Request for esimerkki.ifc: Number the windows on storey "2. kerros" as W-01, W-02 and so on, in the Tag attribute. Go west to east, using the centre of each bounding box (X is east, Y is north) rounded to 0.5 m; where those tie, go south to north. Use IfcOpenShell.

First a look at what the model holds.

```python
import ifcopenshell
import ifcopenshell.util.element
import ifcopenshell.util.placement

model = ifcopenshell.open("esimerkki.ifc")
print(model.schema)
storey = next(s for s in model.by_type("IfcBuildingStorey") if s.Name == "2. kerros")
windows = [e for e in ifcopenshell.util.element.get_decomposition(storey) if e.is_a("IfcWindow")]
for e in sorted(windows, key=lambda e: e.id()):
    origin = ifcopenshell.util.placement.get_local_placement(e.ObjectPlacement)[:3, 3]
    print(e.id(), e.Tag, e.Name, origin.round(2) + 0.0, sep=" | ")
```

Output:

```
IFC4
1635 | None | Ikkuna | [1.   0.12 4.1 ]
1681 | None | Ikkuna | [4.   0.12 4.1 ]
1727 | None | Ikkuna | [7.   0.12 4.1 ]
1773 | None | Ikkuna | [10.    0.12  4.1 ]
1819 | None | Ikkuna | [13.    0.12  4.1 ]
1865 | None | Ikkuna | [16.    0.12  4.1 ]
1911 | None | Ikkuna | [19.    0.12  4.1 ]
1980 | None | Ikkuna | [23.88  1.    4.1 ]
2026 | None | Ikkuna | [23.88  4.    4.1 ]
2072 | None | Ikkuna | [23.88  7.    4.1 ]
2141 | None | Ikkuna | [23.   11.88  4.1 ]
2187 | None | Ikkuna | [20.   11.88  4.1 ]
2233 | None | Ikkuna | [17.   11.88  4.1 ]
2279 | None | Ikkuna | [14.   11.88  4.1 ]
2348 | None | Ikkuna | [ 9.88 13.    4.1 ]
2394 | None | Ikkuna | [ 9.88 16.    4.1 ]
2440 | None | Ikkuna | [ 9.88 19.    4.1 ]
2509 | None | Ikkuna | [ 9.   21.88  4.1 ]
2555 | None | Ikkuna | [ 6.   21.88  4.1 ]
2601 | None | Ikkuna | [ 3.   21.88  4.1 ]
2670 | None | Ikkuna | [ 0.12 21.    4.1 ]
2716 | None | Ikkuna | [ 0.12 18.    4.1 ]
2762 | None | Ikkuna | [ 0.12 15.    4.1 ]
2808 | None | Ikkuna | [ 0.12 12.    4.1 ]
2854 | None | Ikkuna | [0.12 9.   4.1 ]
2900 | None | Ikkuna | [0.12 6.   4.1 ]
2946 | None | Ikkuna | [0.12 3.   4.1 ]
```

```python
import ifcopenshell
import ifcopenshell.geom
import ifcopenshell.util.element
import ifcopenshell.util.shape

model = ifcopenshell.open("esimerkki.ifc")
settings = ifcopenshell.geom.settings()
settings.set("use-world-coords", True)


def centre(element):
    shape = ifcopenshell.geom.create_shape(settings, element)
    return ifcopenshell.util.shape.get_bbox_centroid(shape.geometry)


storey = next(s for s in model.by_type("IfcBuildingStorey") if s.Name == "2. kerros")
windows = [e for e in ifcopenshell.util.element.get_decomposition(storey) if e.is_a("IfcWindow")]

# Insertion points can sit at a corner or the storey origin, so sort by the geometry (in metres).
centres = {e: centre(e) for e in windows}
windows.sort(key=lambda e: (round(centres[e][0] / 0.5), centres[e][1]))

for i, e in enumerate(windows, start=1):
    number = f"W-{i:02d}"
    e.Tag = number
    print(e.id(), number)

model.write("esimerkki_edited.ifc")
```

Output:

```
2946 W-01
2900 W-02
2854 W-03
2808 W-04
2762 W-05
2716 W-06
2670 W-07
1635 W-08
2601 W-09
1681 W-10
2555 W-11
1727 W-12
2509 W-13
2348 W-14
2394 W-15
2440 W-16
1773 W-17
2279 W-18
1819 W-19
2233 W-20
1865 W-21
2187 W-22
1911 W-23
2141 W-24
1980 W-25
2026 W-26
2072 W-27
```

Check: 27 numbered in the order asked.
